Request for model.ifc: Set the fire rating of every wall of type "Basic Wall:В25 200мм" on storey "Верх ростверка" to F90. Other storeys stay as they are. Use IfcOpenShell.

First a look at what the model holds.

```python
import ifcopenshell
import ifcopenshell.util.element

model = ifcopenshell.open("model.ifc")
print(model.schema)
storey = next(s for s in model.by_type("IfcBuildingStorey") if s.Name == "Верх ростверка")
walls = [e for e in ifcopenshell.util.element.get_decomposition(storey) if e.is_a("IfcWall")]
seen = {}
for e in walls:
    element_type = ifcopenshell.util.element.get_type(e)
    key = (element_type.Name if element_type != e and element_type else None, ifcopenshell.util.element.get_pset(e, "Pset_WallCommon", "FireRating"))
    seen[key] = seen.get(key, 0) + 1
for (name, value), count in sorted(seen.items(), key=str):
    print(count, "x", name, "|", value)
```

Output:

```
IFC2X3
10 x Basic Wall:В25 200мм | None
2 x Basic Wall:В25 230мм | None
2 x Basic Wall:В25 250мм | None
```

```python
import ifcopenshell
import ifcopenshell.api.pset
import ifcopenshell.util.element

model = ifcopenshell.open("model.ifc")

storey = next(s for s in model.by_type("IfcBuildingStorey") if s.Name == "Верх ростверка")
walls = [e for e in ifcopenshell.util.element.get_decomposition(storey) if e.is_a("IfcWall")]

count = 0
for e in walls:
    element_type = ifcopenshell.util.element.get_type(e)
    if element_type in (None, e) or element_type.Name != "Basic Wall:В25 200мм":
        continue
    # add_pset returns the element's existing set when there is one.
    pset = ifcopenshell.api.pset.add_pset(model, product=e, name="Pset_WallCommon")
    ifcopenshell.api.pset.edit_pset(model, pset=pset, properties={"FireRating": "F90"})
    count += 1

print(count, "walls updated")

model.write("model_rev.ifc")
```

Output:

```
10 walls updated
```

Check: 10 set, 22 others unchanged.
